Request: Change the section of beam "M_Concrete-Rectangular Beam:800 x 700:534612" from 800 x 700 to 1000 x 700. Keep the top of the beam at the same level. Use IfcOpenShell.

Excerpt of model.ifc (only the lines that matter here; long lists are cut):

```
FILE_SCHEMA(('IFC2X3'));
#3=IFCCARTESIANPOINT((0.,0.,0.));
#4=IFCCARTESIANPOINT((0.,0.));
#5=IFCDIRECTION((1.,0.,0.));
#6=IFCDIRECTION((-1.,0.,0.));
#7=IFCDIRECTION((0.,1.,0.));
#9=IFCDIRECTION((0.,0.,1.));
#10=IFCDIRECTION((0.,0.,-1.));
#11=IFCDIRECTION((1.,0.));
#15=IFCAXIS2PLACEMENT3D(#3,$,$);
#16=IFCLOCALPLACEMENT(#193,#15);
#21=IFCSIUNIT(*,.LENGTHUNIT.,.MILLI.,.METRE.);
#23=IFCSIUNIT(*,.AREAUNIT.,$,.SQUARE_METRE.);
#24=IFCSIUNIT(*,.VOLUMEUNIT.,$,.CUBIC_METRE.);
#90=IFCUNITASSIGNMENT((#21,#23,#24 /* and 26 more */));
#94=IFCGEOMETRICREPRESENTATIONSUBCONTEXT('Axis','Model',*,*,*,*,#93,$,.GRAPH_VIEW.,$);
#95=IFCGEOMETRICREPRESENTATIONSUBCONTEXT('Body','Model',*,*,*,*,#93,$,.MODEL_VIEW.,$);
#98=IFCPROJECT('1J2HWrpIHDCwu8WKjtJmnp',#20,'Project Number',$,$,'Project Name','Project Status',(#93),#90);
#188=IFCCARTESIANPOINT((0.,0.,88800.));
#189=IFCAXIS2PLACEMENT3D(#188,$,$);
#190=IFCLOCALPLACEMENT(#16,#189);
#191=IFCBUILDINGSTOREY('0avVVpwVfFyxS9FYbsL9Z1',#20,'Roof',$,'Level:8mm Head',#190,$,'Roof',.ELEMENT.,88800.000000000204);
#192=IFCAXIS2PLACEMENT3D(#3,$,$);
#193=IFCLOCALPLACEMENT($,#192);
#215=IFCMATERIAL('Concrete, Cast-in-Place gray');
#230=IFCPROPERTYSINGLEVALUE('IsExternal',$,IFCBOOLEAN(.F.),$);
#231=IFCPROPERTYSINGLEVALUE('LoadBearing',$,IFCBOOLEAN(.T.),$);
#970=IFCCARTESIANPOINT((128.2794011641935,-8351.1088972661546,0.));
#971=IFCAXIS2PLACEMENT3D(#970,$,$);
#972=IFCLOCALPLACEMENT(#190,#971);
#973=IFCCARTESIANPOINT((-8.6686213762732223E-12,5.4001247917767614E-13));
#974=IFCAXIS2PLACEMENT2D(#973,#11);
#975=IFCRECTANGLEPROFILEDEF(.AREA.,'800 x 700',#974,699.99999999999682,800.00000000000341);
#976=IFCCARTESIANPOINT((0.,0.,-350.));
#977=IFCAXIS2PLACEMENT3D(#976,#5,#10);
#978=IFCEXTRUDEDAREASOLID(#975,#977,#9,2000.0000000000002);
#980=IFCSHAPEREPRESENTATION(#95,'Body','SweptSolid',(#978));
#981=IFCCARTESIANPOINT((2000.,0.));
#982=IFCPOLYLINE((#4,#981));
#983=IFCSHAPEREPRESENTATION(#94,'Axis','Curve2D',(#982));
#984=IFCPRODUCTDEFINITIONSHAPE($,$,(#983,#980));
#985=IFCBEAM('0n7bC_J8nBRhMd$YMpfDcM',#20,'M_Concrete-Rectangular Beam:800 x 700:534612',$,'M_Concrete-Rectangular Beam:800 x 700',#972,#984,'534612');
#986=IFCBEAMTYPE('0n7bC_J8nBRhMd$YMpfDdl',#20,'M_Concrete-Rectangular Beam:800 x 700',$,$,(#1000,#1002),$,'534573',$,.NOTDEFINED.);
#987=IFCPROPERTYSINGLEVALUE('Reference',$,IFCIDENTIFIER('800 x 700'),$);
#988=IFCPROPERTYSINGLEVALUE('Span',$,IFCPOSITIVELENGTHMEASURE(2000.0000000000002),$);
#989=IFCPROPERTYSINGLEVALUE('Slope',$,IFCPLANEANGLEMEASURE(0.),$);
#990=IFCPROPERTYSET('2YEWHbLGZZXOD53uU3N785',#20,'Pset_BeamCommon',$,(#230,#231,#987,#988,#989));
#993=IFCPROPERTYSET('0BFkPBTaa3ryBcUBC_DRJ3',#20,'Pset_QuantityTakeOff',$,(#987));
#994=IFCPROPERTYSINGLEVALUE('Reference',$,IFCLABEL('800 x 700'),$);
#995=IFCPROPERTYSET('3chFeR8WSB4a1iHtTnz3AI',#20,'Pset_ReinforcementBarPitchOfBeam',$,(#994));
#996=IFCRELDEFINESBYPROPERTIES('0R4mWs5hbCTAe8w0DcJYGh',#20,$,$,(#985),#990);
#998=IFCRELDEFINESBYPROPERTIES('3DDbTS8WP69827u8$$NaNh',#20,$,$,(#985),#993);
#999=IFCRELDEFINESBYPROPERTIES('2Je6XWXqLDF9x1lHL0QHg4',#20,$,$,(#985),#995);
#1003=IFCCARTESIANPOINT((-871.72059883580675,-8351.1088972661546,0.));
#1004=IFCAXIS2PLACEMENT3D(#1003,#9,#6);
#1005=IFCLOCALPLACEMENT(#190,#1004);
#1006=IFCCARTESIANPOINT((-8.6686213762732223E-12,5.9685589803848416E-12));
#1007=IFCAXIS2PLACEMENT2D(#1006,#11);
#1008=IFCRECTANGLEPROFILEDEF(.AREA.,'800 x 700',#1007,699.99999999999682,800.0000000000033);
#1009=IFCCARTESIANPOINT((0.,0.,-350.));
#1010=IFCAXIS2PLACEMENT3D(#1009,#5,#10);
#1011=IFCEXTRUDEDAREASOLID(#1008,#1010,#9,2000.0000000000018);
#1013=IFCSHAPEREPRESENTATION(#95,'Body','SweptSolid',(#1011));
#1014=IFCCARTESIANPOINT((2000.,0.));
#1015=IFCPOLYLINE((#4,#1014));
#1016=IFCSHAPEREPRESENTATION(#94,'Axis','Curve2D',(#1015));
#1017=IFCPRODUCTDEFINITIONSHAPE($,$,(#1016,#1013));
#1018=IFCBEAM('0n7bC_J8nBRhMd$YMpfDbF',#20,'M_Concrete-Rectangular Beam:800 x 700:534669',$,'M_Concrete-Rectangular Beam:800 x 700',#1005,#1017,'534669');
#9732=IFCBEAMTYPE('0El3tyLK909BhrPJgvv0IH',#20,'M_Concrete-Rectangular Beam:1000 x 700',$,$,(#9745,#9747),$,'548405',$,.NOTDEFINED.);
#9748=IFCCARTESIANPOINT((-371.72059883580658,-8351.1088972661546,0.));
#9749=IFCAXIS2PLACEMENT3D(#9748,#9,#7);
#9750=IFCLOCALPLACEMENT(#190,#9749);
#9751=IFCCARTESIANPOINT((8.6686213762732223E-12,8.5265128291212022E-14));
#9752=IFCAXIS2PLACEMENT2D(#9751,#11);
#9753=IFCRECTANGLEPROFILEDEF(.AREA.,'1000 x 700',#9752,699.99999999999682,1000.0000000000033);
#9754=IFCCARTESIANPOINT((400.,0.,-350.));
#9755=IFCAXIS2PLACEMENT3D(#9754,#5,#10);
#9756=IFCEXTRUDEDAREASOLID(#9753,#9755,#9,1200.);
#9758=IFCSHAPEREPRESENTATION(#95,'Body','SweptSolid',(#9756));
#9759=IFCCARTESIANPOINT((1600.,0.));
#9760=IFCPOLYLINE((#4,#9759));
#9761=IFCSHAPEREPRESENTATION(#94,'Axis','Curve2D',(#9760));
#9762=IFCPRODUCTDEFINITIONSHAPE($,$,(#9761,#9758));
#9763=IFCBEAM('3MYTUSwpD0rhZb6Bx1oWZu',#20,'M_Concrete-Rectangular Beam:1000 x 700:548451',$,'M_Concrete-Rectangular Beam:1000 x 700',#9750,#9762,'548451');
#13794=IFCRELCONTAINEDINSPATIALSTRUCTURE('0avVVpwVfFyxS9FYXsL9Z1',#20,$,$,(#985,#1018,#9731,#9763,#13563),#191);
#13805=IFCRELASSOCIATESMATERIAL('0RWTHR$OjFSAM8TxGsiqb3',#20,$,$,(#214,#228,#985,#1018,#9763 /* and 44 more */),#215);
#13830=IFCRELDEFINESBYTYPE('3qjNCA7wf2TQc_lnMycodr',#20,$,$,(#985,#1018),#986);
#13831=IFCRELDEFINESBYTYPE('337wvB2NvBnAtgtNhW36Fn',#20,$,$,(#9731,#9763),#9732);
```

```python
import ifcopenshell
import ifcopenshell.api.pset
import ifcopenshell.api.type
import ifcopenshell.util.element
import ifcopenshell.util.representation

model = ifcopenshell.open("model.ifc")

member = model.by_guid("0n7bC_J8nBRhMd$YMpfDcM")
source = next(p for p in model.by_type("IfcRectangleProfileDef") if p.ProfileName == "1000 x 700")

body = ifcopenshell.util.representation.get_representation(member, "Model", "Body")
solid = body.Items[0]
old_profile = solid.SweptArea

# Copy the section's sizes but keep this member's own profile position.
profile = ifcopenshell.util.element.copy(model, source)
# Profiles are centred, so shift by half the change in depth to hold the top.
shift = (old_profile.XDim - profile.XDim) / 2
x, y = old_profile.Position.Location.Coordinates
up = (-1.0, 0.0)  # upwards, in the solid's own plane
location = model.createIfcCartesianPoint((x + up[0] * shift, y + up[1] * shift))
profile.Position = model.createIfcAxis2Placement2D(location, old_profile.Position.RefDirection)
solid.SweptArea = profile
if not model.get_total_inverses(old_profile):
    ifcopenshell.util.element.remove_deep2(model, old_profile)

new_type = model.by_guid("0El3tyLK909BhrPJgvv0IH")
ifcopenshell.api.type.assign_type(
    model, related_objects=[member], relating_type=new_type, should_map_representations=False
)
member.Name = member.Name.replace("800 x 700", "1000 x 700")
member.ObjectType = "M_Concrete-Rectangular Beam:1000 x 700"
pset = model.by_id(ifcopenshell.util.element.get_pset(member, "Pset_BeamCommon", should_inherit=False)["id"])
ifcopenshell.api.pset.edit_pset(model, pset=pset, properties={"Reference": "1000 x 700"})
pset = model.by_id(ifcopenshell.util.element.get_pset(member, "Pset_QuantityTakeOff", should_inherit=False)["id"])
ifcopenshell.api.pset.edit_pset(model, pset=pset, properties={"Reference": "1000 x 700"})
pset = model.by_id(ifcopenshell.util.element.get_pset(member, "Pset_ReinforcementBarPitchOfBeam", should_inherit=False)["id"])
ifcopenshell.api.pset.edit_pset(model, pset=pset, properties={"Reference": "1000 x 700"})

print(solid.SweptArea)

model.write("model_edited.ifc")
```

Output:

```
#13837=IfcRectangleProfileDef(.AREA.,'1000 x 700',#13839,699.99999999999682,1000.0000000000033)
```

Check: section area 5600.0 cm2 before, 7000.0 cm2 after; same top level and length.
